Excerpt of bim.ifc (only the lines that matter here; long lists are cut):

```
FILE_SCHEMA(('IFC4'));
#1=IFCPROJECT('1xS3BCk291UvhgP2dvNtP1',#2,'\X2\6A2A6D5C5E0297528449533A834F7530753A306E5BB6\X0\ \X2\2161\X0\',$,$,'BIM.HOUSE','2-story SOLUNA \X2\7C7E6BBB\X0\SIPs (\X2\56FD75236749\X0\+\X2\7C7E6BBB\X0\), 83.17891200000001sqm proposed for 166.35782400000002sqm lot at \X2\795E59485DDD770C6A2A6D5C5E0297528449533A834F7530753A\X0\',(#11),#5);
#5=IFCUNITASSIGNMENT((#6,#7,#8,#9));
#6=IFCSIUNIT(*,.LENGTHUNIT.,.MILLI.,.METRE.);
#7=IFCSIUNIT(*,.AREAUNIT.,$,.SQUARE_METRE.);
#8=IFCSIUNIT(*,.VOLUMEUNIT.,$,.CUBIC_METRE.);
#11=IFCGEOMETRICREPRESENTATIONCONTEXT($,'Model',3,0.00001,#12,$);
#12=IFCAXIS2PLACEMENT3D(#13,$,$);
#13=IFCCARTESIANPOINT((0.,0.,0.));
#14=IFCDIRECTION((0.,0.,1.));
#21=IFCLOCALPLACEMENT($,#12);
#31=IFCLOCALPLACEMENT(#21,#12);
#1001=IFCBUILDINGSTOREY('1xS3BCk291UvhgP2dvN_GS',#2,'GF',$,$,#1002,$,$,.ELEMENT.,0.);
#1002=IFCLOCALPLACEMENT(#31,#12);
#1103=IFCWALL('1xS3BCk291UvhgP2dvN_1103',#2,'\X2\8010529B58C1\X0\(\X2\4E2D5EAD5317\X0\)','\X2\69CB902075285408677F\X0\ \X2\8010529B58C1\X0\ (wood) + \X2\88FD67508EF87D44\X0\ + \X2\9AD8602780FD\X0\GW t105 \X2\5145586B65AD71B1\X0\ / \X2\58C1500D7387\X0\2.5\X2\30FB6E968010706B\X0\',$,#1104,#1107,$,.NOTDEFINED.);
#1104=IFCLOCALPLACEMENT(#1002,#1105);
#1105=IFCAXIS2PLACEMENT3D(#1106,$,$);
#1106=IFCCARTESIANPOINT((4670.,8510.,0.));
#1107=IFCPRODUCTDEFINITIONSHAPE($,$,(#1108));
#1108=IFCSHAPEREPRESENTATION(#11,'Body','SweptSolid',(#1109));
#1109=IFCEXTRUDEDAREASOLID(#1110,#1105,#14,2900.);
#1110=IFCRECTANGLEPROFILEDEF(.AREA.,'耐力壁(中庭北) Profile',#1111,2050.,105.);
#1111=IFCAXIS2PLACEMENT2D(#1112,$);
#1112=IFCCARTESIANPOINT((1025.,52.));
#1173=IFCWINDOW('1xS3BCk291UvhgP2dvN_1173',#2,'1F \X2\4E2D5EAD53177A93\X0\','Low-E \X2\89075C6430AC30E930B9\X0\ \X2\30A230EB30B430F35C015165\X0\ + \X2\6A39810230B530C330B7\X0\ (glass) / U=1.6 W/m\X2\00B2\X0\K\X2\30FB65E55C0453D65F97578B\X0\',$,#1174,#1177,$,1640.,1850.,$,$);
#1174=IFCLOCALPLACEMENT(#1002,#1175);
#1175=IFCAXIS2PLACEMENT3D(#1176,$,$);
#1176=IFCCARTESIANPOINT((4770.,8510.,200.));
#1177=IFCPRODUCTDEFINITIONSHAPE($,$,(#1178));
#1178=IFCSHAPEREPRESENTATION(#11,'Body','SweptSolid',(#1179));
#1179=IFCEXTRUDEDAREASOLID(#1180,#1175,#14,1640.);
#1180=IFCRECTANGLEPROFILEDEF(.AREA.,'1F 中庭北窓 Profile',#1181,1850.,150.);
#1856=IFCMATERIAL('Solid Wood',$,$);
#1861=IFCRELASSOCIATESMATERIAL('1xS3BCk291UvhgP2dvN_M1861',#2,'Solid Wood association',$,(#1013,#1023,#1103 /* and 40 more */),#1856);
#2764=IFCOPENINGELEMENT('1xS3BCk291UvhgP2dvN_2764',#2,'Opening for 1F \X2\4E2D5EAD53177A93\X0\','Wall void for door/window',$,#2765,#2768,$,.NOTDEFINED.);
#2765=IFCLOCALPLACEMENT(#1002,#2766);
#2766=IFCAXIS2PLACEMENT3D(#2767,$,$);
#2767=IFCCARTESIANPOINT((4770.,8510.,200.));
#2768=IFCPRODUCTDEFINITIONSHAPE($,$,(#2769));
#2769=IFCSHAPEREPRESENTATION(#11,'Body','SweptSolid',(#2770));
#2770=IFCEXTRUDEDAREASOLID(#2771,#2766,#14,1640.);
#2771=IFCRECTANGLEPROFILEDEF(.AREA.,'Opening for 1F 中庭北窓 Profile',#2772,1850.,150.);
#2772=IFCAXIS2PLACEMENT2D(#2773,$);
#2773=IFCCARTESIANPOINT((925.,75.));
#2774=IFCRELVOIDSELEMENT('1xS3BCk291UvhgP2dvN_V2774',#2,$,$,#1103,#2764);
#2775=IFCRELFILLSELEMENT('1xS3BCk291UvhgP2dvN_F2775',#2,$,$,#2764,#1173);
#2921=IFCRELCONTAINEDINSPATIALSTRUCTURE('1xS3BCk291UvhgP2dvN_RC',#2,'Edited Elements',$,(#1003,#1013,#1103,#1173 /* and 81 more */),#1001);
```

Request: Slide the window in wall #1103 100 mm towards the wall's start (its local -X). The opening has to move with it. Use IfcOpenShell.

```python
import ifcopenshell
import ifcopenshell.api.geometry
import ifcopenshell.util.placement
import ifcopenshell.util.unit

model = ifcopenshell.open("bim.ifc")
unit_scale = ifcopenshell.util.unit.calculate_unit_scale(model)

window = model.by_id(1173)
opening = window.FillsVoids[0].RelatingOpeningElement
wall = opening.VoidsElements[0].RelatingBuildingElement

wall_matrix = ifcopenshell.util.placement.get_local_placement(wall.ObjectPlacement)
shift = wall_matrix[:3, 0] * -0.1 / unit_scale
before = ifcopenshell.util.placement.get_local_placement(window.ObjectPlacement)[:3, 3].copy()

# The window is not placed relative to its opening, so move both.
for product in (opening, window):
    matrix = ifcopenshell.util.placement.get_local_placement(product.ObjectPlacement)
    matrix[:3, 3] += shift
    ifcopenshell.api.geometry.edit_object_placement(model, product=product, matrix=matrix, is_si=False)

after = ifcopenshell.util.placement.get_local_placement(window.ObjectPlacement)[:3, 3]
print("window moved by", (after - before).round(3) + 0.0)

model.write("bim_edited.ifc")
```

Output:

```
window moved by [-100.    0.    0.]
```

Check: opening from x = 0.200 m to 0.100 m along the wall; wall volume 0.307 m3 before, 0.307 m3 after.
